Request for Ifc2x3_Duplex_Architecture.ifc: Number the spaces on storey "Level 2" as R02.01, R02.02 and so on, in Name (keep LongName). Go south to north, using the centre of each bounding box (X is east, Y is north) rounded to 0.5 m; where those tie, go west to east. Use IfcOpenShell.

First a look at what the model holds.

```python
import ifcopenshell
import ifcopenshell.util.element
import ifcopenshell.util.placement

model = ifcopenshell.open("Ifc2x3_Duplex_Architecture.ifc")
print(model.schema)
storey = next(s for s in model.by_type("IfcBuildingStorey") if s.Name == "Level 2")
spaces = [e for e in ifcopenshell.util.element.get_decomposition(storey) if e.is_a("IfcSpace")]
for e in sorted(spaces, key=lambda e: e.id()):
    origin = ifcopenshell.util.placement.get_local_placement(e.ObjectPlacement)[:3, 3]
    print(e.id(), e.Name, e.LongName, origin.round(2) + 0.0, sep=" | ")
```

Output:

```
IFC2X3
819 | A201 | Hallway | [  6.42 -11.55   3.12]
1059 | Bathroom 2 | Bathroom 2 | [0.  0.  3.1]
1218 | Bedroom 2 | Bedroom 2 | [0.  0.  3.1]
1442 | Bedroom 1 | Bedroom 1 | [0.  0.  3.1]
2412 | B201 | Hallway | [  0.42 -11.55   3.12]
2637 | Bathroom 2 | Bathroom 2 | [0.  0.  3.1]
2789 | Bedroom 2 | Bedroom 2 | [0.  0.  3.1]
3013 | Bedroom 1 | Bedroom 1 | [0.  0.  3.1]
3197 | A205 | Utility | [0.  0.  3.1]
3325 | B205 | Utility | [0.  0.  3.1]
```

```python
import ifcopenshell
import ifcopenshell.geom
import ifcopenshell.util.element
import ifcopenshell.util.shape

model = ifcopenshell.open("Ifc2x3_Duplex_Architecture.ifc")
settings = ifcopenshell.geom.settings()
settings.set("use-world-coords", True)


def centre(element):
    shape = ifcopenshell.geom.create_shape(settings, element)
    return ifcopenshell.util.shape.get_bbox_centroid(shape.geometry)


storey = next(s for s in model.by_type("IfcBuildingStorey") if s.Name == "Level 2")
spaces = [e for e in ifcopenshell.util.element.get_decomposition(storey) if e.is_a("IfcSpace")]

# Insertion points can sit at a corner or the storey origin, so sort by the geometry (in metres).
centres = {e: centre(e) for e in spaces}
spaces.sort(key=lambda e: (round(centres[e][1] / 0.5), centres[e][0]))

for i, e in enumerate(spaces, start=1):
    number = f"R02.{i:02d}"
    e.Name = number
    print(e.id(), number)

model.write("Ifc2x3_Duplex_Architecture_edited.ifc")
```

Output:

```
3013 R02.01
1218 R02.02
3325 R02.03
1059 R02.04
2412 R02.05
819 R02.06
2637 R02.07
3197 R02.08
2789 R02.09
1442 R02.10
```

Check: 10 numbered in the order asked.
